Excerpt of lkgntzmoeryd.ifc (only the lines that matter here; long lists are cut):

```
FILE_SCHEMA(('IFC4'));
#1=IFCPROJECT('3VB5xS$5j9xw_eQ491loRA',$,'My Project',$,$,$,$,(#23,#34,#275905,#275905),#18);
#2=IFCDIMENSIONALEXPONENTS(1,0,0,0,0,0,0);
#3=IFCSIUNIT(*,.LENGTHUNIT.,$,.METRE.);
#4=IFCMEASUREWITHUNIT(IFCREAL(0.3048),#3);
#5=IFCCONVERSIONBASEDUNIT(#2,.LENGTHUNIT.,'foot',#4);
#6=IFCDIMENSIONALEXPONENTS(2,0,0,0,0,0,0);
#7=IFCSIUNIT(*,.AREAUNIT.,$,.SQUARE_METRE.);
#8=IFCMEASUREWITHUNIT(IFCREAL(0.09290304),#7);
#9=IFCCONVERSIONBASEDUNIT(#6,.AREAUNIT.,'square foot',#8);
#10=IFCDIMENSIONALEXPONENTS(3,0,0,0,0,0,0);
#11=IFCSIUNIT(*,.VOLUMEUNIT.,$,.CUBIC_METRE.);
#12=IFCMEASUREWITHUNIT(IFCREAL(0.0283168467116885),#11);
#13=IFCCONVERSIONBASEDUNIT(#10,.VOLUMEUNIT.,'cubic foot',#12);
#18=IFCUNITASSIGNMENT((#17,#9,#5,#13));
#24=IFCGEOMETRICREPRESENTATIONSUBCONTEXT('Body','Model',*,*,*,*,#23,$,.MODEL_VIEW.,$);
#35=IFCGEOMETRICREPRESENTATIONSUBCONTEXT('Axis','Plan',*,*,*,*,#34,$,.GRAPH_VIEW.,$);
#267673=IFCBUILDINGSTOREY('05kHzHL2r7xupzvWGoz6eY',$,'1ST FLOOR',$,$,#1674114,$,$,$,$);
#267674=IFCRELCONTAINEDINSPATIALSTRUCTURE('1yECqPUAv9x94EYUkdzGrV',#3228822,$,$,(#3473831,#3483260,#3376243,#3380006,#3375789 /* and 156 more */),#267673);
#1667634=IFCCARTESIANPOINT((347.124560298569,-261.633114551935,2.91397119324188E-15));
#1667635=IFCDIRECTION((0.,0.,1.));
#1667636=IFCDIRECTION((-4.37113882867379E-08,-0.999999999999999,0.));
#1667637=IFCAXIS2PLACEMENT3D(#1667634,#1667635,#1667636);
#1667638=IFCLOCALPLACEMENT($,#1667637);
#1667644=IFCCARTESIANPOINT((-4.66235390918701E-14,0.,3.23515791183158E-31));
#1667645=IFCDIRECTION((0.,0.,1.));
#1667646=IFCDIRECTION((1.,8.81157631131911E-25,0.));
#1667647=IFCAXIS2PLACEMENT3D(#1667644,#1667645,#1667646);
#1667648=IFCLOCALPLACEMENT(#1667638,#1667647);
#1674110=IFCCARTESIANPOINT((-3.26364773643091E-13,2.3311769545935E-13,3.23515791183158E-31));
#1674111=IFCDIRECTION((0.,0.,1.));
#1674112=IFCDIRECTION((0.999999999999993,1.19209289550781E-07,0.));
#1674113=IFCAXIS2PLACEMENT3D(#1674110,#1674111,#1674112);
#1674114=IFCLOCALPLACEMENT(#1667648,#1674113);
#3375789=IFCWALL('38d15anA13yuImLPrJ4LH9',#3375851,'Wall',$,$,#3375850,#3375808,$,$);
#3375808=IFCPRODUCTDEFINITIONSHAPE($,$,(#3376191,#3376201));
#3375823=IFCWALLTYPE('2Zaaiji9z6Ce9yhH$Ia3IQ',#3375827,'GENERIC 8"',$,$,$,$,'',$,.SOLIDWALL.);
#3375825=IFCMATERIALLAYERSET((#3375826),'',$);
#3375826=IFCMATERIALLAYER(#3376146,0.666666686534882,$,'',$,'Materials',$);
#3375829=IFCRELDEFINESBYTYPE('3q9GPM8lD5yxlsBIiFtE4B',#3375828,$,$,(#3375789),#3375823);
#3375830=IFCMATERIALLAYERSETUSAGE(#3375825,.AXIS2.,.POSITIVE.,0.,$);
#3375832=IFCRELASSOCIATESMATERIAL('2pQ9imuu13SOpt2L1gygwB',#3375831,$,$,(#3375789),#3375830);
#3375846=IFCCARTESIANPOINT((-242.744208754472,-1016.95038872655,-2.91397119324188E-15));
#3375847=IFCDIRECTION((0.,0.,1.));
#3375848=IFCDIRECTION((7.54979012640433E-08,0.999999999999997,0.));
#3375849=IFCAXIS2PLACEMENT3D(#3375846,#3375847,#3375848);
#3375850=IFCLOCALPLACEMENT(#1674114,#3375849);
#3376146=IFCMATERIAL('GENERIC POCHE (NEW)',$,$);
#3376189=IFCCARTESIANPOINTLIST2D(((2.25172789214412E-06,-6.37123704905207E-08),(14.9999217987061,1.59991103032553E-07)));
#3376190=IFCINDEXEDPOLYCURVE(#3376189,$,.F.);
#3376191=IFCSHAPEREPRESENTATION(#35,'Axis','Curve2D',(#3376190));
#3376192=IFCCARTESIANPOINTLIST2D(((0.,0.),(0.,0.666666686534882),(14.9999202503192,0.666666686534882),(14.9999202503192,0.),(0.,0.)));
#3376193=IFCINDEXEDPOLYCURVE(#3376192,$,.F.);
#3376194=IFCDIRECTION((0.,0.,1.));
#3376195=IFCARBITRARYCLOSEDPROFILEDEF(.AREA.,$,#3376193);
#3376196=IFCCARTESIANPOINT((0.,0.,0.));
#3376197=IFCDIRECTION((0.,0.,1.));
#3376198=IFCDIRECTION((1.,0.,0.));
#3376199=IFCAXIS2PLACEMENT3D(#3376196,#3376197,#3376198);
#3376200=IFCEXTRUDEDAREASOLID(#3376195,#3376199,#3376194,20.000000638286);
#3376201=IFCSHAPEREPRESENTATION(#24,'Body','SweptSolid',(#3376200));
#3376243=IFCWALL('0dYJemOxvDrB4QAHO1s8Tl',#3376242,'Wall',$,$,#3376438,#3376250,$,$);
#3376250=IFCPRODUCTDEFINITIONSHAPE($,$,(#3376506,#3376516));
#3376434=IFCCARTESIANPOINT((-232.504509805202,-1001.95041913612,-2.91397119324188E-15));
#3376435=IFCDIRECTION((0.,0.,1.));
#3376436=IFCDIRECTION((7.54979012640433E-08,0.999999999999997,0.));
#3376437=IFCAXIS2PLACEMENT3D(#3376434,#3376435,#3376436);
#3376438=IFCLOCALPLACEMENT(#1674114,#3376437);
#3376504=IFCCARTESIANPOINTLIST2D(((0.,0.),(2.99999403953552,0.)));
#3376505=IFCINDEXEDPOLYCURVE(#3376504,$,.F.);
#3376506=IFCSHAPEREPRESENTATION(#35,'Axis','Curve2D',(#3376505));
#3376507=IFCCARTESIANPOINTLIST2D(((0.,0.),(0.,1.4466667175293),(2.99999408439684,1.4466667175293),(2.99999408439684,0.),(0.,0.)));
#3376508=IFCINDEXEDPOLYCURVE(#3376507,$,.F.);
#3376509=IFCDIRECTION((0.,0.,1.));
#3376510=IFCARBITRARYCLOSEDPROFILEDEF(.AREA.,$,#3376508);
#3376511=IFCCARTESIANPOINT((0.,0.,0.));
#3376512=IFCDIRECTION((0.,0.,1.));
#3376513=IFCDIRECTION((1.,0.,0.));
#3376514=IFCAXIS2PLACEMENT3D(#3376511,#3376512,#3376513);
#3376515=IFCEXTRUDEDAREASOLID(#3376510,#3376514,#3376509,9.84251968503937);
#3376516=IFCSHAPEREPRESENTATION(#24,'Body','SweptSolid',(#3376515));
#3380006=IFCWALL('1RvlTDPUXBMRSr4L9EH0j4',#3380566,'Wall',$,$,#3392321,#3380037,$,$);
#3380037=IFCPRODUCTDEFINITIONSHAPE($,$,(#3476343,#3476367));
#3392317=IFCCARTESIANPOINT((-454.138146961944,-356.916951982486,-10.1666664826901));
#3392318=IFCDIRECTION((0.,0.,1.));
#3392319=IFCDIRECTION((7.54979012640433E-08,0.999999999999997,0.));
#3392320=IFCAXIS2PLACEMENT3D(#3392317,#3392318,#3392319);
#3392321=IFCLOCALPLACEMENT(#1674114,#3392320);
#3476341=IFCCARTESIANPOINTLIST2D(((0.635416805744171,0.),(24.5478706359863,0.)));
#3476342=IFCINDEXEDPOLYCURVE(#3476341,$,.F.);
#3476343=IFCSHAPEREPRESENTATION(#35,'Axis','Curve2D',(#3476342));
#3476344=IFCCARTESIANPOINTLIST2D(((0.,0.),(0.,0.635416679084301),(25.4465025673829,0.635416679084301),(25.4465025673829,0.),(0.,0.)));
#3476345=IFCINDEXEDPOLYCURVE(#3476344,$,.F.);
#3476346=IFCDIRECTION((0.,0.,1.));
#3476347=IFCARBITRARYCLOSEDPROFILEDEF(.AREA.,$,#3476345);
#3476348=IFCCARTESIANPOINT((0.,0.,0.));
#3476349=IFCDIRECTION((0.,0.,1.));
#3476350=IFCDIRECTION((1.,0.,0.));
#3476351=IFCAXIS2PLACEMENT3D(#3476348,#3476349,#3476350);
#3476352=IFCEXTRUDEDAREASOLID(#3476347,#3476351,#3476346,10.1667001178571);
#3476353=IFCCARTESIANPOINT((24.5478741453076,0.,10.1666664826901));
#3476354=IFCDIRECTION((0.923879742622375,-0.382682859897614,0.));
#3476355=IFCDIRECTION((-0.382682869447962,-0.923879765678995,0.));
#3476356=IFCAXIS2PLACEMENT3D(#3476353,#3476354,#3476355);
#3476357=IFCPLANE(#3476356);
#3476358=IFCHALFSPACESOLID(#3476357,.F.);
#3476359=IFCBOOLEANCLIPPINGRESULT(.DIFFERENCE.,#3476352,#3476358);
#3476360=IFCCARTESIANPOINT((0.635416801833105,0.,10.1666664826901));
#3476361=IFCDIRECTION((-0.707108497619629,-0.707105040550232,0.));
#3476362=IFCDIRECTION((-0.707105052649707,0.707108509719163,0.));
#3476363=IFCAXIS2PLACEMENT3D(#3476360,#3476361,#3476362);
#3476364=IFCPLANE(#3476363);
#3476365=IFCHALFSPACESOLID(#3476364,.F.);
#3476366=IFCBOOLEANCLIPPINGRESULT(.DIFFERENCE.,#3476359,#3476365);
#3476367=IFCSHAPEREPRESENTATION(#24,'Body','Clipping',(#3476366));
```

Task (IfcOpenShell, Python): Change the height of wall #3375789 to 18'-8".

```python
import ifcopenshell
import ifcopenshell.geom
import ifcopenshell.util.representation
import ifcopenshell.util.shape
import ifcopenshell.util.unit

model = ifcopenshell.open("lkgntzmoeryd.ifc")
unit_scale = ifcopenshell.util.unit.calculate_unit_scale(model)
settings = ifcopenshell.geom.settings()


def volume(element):
    """Net volume in cubic metres, openings subtracted."""
    shape = ifcopenshell.geom.create_shape(settings, element)
    return ifcopenshell.util.shape.get_volume(shape.geometry)


wall = model.by_id(3375789)
before = volume(wall)

body = ifcopenshell.util.representation.get_representation(wall, "Model", "Body")
solid = body.Items[0]
old_height = solid.Depth
solid.Depth = 224 * 0.0254 / unit_scale
after = volume(wall)

print(f"height {old_height:g} -> {solid.Depth:g}, volume {before:.3f} -> {after:.3f} m3")

model.write("lkgntzmoeryd_rev.ifc")
```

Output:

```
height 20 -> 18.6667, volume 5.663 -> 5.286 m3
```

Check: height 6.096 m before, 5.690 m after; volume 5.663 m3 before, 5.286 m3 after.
